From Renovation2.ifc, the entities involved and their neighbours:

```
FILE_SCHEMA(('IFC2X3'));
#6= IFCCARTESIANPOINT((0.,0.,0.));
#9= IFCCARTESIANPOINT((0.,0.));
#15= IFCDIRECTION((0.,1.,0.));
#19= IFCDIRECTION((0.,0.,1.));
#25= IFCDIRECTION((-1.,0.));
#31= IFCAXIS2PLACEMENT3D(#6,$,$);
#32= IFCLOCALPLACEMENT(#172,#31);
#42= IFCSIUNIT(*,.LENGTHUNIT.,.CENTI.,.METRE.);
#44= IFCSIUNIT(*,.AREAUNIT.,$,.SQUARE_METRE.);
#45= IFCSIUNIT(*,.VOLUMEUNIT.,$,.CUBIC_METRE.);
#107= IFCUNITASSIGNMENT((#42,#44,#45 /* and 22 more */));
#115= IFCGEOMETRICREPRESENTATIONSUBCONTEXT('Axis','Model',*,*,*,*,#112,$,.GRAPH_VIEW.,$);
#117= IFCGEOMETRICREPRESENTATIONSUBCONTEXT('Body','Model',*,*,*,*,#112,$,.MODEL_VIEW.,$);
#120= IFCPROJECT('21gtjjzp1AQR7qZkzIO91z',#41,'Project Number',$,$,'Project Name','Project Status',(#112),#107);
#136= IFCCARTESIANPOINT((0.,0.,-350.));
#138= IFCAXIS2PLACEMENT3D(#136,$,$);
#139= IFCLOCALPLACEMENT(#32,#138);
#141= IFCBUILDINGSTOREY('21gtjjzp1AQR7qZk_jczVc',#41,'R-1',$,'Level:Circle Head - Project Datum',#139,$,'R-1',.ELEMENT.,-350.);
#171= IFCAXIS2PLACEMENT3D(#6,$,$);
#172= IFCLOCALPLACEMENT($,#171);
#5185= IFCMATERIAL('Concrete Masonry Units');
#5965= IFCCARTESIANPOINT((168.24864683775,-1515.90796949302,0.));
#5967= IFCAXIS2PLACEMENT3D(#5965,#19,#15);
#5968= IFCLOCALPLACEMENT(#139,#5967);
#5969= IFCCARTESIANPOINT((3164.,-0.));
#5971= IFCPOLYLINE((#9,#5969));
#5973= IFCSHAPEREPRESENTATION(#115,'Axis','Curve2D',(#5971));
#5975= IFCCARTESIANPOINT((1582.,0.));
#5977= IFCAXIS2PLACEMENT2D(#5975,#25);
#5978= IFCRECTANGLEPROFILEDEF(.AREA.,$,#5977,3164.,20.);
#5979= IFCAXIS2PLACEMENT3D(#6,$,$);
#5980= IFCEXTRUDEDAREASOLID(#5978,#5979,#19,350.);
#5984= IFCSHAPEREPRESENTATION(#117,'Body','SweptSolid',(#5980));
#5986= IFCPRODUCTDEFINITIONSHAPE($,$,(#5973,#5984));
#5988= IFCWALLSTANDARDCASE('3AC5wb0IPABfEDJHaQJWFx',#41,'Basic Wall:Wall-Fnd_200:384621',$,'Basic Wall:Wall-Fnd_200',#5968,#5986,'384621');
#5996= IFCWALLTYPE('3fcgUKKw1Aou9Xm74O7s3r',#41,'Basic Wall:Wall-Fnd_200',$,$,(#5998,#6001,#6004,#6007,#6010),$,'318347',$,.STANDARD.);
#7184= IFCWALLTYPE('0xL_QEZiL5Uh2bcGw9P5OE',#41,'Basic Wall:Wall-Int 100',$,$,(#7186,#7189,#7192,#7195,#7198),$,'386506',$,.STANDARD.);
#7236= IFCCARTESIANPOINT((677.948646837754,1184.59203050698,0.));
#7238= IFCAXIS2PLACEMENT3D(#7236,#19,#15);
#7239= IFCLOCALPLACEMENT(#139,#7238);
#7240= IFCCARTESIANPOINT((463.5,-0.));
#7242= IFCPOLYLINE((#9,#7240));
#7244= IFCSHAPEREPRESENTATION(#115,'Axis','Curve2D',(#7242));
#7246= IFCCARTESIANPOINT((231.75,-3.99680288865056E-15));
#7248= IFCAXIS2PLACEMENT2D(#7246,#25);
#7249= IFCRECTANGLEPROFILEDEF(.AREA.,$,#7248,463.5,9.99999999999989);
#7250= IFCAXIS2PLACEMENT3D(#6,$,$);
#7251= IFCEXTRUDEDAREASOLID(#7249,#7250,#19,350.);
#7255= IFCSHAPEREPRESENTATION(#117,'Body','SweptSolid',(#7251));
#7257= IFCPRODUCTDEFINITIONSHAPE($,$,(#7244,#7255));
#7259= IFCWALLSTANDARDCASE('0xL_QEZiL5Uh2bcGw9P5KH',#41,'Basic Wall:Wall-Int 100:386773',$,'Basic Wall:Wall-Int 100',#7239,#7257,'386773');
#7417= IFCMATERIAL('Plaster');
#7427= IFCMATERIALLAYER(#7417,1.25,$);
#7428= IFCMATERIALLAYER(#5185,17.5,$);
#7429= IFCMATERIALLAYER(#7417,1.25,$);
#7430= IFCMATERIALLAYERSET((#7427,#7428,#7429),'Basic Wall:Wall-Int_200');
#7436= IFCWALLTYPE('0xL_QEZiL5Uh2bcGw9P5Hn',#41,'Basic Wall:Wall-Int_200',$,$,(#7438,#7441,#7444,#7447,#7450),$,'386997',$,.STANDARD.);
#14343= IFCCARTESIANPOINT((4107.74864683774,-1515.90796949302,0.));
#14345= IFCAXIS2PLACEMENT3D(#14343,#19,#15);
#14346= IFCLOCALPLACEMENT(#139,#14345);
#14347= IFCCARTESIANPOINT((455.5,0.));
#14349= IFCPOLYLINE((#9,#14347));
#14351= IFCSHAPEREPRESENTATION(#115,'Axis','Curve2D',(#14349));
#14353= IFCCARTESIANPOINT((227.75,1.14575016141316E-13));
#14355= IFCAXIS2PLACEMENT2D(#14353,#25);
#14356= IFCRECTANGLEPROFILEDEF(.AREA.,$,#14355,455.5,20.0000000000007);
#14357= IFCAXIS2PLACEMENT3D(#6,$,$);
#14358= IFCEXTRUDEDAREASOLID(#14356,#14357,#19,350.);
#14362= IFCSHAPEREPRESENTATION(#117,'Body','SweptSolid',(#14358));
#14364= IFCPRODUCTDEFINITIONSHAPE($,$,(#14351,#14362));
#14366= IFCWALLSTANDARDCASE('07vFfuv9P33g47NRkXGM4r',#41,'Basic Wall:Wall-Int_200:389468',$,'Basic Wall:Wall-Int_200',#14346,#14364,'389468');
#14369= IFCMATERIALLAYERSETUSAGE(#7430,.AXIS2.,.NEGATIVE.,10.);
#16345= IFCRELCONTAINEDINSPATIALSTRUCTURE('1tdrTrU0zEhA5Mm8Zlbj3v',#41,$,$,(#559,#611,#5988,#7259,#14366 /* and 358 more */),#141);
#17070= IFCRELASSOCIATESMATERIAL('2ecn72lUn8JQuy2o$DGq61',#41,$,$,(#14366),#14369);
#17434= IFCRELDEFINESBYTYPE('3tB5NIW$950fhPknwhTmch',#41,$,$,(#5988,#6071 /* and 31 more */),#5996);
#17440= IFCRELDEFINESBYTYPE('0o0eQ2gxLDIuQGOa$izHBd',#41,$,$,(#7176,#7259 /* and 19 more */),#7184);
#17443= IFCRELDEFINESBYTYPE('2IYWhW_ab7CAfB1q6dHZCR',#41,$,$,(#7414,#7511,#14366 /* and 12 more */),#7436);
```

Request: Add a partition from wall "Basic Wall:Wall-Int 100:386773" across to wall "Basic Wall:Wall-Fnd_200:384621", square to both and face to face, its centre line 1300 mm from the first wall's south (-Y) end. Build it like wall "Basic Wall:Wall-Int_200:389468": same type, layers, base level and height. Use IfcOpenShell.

```python
import numpy as np
import ifcopenshell
import ifcopenshell.api.geometry
import ifcopenshell.api.material
import ifcopenshell.api.pset
import ifcopenshell.api.root
import ifcopenshell.api.spatial
import ifcopenshell.api.type
import ifcopenshell.geom
import ifcopenshell.util.element
import ifcopenshell.util.placement
import ifcopenshell.util.representation
import ifcopenshell.util.shape
import ifcopenshell.util.unit

model = ifcopenshell.open("Renovation2.ifc")
unit_scale = ifcopenshell.util.unit.calculate_unit_scale(model)
settings = ifcopenshell.geom.settings()
settings.set("use-world-coords", True)

start_wall = model.by_id(7259)
end_wall = model.by_guid("3AC5wb0IPABfEDJHaQJWFx")
like = model.by_guid("07vFfuv9P33g47NRkXGM4r")
matrix = ifcopenshell.util.placement.get_local_placement(start_wall.ObjectPlacement)
matrix[:3, 3] *= unit_scale


def extent(element):
    """Bounding box in the first wall's axes, in metres."""
    shape = ifcopenshell.geom.create_shape(settings, element)
    points = (ifcopenshell.util.shape.get_vertices(shape.geometry) - matrix[:3, 3]) @ matrix[:3, :3]
    return points.min(axis=0), points.max(axis=0)


y_start = extent(start_wall)[1][1]
y_end = extent(end_wall)[0][1]
like_min, like_max = extent(like)
length, height = float(abs(y_end - y_start)), float(like_max[2] - like_min[2])
layer_set = ifcopenshell.util.element.get_material(like, should_skip_usage=True)
thickness = sum(layer.LayerThickness for layer in layer_set.MaterialLayers) * unit_scale

wall = ifcopenshell.api.root.create_entity(model, ifc_class="IfcWallStandardCase", name="New partition")
storey = ifcopenshell.util.element.get_container(like)
ifcopenshell.api.spatial.assign_container(model, products=[wall], relating_structure=storey)
ifcopenshell.api.type.assign_type(
    model, related_objects=[wall], relating_type=ifcopenshell.util.element.get_type(like), should_map_representations=False
)
rel = ifcopenshell.api.material.assign_material(
    model, products=[wall], type="IfcMaterialLayerSetUsage", material=layer_set
)
rel.RelatingMaterial.OffsetFromReferenceLine = -thickness / 2 / unit_scale
pset = ifcopenshell.api.pset.add_pset(model, product=wall, name="Pset_WallCommon")
ifcopenshell.api.pset.edit_pset(model, pset=pset, properties={"IsExternal": False, "LoadBearing": False})

# The axis runs down the middle of the wall.
axis = ifcopenshell.api.geometry.add_axis_representation(
    model, context=ifcopenshell.util.representation.get_context(model, "Model", "Axis"), axis=[(0.0, 0.0), (length, 0.0)]
)
body = ifcopenshell.api.geometry.add_wall_representation(
    model,
    context=ifcopenshell.util.representation.get_context(model, "Model", "Body", "MODEL_VIEW"),
    length=length,
    height=height,
    thickness=thickness,
    offset=-thickness / 2,
)
for representation in (axis, body):
    ifcopenshell.api.geometry.assign_representation(model, product=wall, representation=representation)

placement = matrix @ ifcopenshell.util.placement.rotation(90, "Z")
placement[:, 3] = matrix @ np.array([extent(start_wall)[0][0] + 1.3, y_start, like_min[2], 1.0])
ifcopenshell.api.geometry.edit_object_placement(model, product=wall, matrix=placement)

print(f"partition {length:.3f} m long, {height:.3f} m high, {thickness:.3f} m thick")

model.write("Renovation2_updated.ifc")
```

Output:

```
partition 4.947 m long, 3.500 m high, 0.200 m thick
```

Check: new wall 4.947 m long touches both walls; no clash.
